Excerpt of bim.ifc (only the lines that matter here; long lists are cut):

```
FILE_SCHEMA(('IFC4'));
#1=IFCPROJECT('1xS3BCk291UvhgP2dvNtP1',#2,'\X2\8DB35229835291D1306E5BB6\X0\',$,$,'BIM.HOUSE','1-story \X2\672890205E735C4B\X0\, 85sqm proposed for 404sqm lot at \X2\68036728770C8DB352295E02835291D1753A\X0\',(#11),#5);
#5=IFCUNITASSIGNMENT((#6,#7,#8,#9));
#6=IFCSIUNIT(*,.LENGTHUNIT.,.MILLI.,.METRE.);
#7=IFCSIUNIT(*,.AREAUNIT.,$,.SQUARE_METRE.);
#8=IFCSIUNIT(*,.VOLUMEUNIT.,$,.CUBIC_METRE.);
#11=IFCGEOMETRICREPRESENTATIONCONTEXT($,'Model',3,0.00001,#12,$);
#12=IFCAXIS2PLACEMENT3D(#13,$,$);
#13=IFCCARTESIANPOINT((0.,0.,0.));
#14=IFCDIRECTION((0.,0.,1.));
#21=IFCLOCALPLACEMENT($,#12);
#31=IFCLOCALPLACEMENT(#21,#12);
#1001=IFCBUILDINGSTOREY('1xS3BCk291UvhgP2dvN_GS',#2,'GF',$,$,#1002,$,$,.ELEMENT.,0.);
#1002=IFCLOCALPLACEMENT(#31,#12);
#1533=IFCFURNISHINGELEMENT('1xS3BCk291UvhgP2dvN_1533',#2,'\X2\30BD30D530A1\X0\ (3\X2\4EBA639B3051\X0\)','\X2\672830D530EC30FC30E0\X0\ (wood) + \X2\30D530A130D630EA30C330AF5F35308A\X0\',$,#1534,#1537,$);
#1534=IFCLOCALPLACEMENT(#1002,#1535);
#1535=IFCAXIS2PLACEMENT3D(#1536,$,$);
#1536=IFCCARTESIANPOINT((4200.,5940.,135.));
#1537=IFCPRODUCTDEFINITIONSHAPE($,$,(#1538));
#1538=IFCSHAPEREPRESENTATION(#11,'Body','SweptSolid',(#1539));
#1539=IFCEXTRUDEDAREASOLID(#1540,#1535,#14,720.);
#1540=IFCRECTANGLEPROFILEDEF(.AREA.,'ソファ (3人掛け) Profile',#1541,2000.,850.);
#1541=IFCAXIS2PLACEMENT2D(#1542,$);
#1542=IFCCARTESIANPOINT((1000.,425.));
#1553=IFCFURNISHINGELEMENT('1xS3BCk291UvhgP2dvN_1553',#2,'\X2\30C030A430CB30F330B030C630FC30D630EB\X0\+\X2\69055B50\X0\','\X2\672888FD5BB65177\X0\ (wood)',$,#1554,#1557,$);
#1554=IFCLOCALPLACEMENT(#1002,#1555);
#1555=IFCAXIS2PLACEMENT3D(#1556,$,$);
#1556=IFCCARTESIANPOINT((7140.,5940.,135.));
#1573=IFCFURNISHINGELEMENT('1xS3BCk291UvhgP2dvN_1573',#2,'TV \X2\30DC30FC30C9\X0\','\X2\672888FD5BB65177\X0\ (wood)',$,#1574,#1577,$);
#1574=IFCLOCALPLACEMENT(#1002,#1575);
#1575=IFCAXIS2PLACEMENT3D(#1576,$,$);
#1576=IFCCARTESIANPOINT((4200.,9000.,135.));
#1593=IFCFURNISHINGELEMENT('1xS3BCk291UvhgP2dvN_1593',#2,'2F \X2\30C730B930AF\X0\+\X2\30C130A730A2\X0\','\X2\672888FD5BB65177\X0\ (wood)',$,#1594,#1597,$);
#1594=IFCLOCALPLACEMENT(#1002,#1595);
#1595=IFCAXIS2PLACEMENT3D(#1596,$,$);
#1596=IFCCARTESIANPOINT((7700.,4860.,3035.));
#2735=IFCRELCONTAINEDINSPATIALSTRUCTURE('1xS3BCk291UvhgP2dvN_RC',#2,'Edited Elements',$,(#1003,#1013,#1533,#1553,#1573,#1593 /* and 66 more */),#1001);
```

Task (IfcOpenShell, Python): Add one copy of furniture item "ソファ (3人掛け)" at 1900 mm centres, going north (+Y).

```python
import numpy as np
import ifcopenshell
import ifcopenshell.api.geometry
import ifcopenshell.api.root
import ifcopenshell.util.element
import ifcopenshell.util.placement
import ifcopenshell.util.unit

model = ifcopenshell.open("bim.ifc")
unit_scale = ifcopenshell.util.unit.calculate_unit_scale(model)


def reuse_history(source, copy):
    """copy_class also copies each property set's owner history, people and application; keep the originals."""
    for rel in copy.IsDefinedBy:
        if rel.is_a("IfcRelDefinesByProperties") and (history := rel.RelatingPropertyDefinition.OwnerHistory):
            rel.RelatingPropertyDefinition.OwnerHistory = source.OwnerHistory
            ifcopenshell.util.element.remove_deep2(model, history)


source = model.by_id(1533)
base = ifcopenshell.util.placement.get_local_placement(source.ObjectPlacement)
step = np.array([0.0, 1.0, 0.0]) * 1.9 / unit_scale

for i in range(1, 2):
    copy = ifcopenshell.api.root.copy_class(model, product=source)
    copy.Representation = ifcopenshell.util.element.copy_deep(
        model, source.Representation, exclude=["IfcGeometricRepresentationContext", "IfcRepresentationMap"]
    )
    reuse_history(source, copy)
    matrix = base.copy()
    matrix[:3, 3] += i * step
    print("added at", matrix[:3, 3].round(3) + 0.0)
    ifcopenshell.api.geometry.edit_object_placement(model, product=copy, matrix=matrix, is_si=False)

model.write("bim_v2.ifc")
```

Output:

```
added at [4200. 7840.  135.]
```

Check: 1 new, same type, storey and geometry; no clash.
